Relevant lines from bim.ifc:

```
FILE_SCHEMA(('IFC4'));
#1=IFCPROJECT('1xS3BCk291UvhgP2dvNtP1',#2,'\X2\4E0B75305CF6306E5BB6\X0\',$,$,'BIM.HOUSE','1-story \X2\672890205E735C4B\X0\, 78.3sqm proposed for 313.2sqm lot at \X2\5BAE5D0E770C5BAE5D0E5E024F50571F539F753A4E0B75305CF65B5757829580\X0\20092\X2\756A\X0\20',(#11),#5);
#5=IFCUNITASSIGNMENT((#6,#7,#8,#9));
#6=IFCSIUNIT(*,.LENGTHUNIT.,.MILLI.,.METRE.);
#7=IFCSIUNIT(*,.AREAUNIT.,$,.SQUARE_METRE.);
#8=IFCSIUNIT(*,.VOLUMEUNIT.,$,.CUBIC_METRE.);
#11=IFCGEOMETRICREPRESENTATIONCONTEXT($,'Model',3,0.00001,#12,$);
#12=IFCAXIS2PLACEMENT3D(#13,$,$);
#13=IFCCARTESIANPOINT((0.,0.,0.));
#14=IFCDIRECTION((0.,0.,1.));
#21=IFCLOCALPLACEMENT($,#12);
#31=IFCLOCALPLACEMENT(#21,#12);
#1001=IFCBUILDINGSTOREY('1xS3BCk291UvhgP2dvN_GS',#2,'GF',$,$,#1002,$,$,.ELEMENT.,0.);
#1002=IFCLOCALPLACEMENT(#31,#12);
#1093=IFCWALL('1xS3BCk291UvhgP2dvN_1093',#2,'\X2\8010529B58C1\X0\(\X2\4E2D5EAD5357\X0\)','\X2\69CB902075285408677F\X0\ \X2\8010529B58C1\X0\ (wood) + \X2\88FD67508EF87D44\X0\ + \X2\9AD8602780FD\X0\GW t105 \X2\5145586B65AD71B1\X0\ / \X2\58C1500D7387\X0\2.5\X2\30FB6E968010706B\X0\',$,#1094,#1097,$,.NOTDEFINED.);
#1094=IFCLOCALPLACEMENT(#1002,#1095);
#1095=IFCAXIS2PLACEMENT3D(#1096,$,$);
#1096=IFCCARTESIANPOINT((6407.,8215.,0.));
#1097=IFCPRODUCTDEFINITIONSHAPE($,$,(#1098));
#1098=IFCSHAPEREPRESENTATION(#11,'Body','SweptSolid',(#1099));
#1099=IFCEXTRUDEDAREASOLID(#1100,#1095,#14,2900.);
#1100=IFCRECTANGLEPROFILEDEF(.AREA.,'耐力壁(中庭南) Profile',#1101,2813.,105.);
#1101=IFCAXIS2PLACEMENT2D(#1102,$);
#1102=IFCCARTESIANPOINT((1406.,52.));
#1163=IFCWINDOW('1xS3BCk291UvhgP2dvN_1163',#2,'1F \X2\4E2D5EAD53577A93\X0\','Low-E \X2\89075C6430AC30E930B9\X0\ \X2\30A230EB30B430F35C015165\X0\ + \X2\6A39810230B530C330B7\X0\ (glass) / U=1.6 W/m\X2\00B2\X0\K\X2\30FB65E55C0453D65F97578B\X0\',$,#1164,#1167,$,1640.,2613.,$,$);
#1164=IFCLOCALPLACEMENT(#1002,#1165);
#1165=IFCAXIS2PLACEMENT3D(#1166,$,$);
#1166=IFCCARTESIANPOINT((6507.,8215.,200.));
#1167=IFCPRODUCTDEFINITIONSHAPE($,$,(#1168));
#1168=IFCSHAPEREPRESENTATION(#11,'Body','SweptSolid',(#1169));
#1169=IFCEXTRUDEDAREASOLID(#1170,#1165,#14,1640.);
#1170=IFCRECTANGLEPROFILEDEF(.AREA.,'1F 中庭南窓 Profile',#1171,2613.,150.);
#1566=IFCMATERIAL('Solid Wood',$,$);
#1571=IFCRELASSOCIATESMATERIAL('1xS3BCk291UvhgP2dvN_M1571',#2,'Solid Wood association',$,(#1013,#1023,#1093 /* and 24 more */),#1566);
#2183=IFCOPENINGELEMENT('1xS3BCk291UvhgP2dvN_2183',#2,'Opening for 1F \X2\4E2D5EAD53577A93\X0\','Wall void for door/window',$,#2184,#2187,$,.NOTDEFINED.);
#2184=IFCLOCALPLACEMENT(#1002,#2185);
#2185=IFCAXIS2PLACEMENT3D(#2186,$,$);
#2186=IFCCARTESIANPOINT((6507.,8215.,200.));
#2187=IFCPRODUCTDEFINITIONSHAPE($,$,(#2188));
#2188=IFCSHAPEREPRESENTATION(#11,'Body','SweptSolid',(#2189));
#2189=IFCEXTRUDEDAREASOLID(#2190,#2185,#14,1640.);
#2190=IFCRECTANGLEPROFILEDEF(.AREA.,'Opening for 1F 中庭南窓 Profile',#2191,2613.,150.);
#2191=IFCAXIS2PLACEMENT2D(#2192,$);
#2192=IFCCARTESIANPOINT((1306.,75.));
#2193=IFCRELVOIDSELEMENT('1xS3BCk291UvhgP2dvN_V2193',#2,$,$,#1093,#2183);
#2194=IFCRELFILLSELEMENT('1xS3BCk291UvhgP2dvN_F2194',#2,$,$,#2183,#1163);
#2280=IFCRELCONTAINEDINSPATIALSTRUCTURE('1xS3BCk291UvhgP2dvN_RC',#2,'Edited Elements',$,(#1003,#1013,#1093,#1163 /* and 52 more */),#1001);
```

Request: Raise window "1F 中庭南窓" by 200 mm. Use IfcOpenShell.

```python
import numpy as np
import ifcopenshell
import ifcopenshell.api.geometry
import ifcopenshell.util.placement
import ifcopenshell.util.unit

model = ifcopenshell.open("bim.ifc")
unit_scale = ifcopenshell.util.unit.calculate_unit_scale(model)

window = model.by_guid("1xS3BCk291UvhgP2dvN_1163")
opening = window.FillsVoids[0].RelatingOpeningElement
dz = 0.2 / unit_scale

shift = np.array([0.0, 0.0, dz])
# The window is not placed relative to its opening, so move both.
for product in (opening, window):
    matrix = ifcopenshell.util.placement.get_local_placement(product.ObjectPlacement)
    matrix[:3, 3] += shift
    ifcopenshell.api.geometry.edit_object_placement(model, product=product, matrix=matrix, is_si=False)

print(f"moved by {dz * unit_scale:+.3f} m")

model.write("bim_rev.ifc")
```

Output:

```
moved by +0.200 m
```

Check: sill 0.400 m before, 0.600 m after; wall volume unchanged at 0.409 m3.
